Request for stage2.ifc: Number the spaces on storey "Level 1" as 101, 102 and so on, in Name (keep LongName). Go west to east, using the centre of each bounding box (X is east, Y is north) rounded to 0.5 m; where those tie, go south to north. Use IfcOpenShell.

First a look at what the model holds.

```python
import ifcopenshell
import ifcopenshell.util.element
import ifcopenshell.util.placement

model = ifcopenshell.open("stage2.ifc")
print(model.schema)
storey = next(s for s in model.by_type("IfcBuildingStorey") if s.Name == "Level 1")
spaces = [e for e in ifcopenshell.util.element.get_decomposition(storey) if e.is_a("IfcSpace")]
for e in sorted(spaces, key=lambda e: e.id()):
    origin = ifcopenshell.util.placement.get_local_placement(e.ObjectPlacement)[:3, 3]
    print(e.id(), e.Name, e.LongName, origin.round(2) + 0.0, sep=" | ")
```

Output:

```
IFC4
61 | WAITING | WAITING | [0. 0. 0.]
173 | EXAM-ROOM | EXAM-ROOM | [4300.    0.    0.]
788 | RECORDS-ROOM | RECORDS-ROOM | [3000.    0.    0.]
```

```python
import ifcopenshell
import ifcopenshell.geom
import ifcopenshell.util.element
import ifcopenshell.util.shape

model = ifcopenshell.open("stage2.ifc")
settings = ifcopenshell.geom.settings()
settings.set("use-world-coords", True)


def centre(element):
    shape = ifcopenshell.geom.create_shape(settings, element)
    return ifcopenshell.util.shape.get_bbox_centroid(shape.geometry)


storey = next(s for s in model.by_type("IfcBuildingStorey") if s.Name == "Level 1")
spaces = [e for e in ifcopenshell.util.element.get_decomposition(storey) if e.is_a("IfcSpace")]

# Insertion points can sit at a corner or the storey origin, so sort by the geometry (in metres).
centres = {e: centre(e) for e in spaces}
spaces.sort(key=lambda e: (round(centres[e][0] / 0.5), centres[e][1]))

for i, e in enumerate(spaces, start=1):
    number = f"1{i:02d}"
    e.Name = number
    print(e.id(), number)

model.write("stage2-out.ifc")
```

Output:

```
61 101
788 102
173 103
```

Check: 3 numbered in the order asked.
